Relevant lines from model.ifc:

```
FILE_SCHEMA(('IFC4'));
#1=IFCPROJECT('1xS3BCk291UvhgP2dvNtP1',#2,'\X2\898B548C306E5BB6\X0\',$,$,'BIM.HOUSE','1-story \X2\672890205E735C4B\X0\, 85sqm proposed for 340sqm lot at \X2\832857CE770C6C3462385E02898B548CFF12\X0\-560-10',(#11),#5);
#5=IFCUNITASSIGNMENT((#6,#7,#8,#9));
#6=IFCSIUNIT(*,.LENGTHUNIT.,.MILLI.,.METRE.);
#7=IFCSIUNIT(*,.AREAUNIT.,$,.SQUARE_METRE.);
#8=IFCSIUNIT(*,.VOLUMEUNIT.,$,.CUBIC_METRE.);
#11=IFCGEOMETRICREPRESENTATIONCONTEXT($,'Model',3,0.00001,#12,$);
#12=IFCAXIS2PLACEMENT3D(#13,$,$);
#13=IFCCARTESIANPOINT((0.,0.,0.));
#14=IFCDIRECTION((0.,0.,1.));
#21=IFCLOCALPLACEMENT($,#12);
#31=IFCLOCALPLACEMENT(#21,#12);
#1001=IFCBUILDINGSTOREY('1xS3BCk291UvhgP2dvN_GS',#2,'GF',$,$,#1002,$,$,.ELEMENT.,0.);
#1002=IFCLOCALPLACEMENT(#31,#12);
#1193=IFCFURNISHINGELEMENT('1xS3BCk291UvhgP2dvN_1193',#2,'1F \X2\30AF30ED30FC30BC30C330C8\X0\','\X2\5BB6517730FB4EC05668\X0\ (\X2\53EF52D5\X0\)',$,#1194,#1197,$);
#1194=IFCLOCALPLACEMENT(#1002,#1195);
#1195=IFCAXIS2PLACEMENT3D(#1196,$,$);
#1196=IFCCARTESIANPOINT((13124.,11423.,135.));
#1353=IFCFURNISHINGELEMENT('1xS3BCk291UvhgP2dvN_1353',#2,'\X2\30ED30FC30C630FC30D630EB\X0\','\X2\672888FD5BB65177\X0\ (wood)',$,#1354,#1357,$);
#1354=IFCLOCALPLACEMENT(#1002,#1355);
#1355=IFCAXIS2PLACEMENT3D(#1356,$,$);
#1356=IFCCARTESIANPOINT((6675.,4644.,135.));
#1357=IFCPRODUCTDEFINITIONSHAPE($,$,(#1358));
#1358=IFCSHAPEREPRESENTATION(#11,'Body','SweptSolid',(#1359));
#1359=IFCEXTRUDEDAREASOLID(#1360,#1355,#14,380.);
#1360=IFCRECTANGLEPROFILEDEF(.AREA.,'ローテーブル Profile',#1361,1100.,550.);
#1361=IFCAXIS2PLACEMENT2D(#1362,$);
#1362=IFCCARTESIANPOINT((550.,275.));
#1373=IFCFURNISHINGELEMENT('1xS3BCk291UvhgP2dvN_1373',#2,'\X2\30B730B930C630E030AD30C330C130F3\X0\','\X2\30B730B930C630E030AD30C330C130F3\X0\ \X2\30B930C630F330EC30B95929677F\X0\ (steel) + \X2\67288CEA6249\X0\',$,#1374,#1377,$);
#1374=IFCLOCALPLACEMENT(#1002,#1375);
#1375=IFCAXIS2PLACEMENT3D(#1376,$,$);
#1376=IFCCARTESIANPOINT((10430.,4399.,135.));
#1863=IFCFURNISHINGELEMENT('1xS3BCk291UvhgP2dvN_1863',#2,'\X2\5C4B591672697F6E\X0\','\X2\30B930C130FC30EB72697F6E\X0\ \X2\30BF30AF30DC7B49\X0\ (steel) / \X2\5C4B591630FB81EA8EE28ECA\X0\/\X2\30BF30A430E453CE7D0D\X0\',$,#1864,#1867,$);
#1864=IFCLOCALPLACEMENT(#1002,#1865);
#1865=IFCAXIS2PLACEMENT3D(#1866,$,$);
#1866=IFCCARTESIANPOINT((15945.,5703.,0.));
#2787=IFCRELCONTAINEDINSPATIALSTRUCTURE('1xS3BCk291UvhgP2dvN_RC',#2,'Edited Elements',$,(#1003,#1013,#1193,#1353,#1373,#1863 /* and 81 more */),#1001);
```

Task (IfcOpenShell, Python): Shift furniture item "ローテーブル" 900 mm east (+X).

```python
import ifcopenshell
import ifcopenshell.api.geometry
import ifcopenshell.util.placement

model = ifcopenshell.open("model.ifc")

item = model.by_guid("1xS3BCk291UvhgP2dvN_1353")
matrix = ifcopenshell.util.placement.get_local_placement(item.ObjectPlacement)
matrix[0, 3] += 900.0
ifcopenshell.api.geometry.edit_object_placement(model, product=item, matrix=matrix, is_si=False)

print(ifcopenshell.util.placement.get_local_placement(item.ObjectPlacement).round(3) + 0.0)

model.write("model-out.ifc")
```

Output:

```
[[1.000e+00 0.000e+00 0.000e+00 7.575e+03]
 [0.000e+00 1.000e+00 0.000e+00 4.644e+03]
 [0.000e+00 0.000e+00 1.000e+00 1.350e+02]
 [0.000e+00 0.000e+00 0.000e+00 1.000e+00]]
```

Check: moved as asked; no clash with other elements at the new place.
